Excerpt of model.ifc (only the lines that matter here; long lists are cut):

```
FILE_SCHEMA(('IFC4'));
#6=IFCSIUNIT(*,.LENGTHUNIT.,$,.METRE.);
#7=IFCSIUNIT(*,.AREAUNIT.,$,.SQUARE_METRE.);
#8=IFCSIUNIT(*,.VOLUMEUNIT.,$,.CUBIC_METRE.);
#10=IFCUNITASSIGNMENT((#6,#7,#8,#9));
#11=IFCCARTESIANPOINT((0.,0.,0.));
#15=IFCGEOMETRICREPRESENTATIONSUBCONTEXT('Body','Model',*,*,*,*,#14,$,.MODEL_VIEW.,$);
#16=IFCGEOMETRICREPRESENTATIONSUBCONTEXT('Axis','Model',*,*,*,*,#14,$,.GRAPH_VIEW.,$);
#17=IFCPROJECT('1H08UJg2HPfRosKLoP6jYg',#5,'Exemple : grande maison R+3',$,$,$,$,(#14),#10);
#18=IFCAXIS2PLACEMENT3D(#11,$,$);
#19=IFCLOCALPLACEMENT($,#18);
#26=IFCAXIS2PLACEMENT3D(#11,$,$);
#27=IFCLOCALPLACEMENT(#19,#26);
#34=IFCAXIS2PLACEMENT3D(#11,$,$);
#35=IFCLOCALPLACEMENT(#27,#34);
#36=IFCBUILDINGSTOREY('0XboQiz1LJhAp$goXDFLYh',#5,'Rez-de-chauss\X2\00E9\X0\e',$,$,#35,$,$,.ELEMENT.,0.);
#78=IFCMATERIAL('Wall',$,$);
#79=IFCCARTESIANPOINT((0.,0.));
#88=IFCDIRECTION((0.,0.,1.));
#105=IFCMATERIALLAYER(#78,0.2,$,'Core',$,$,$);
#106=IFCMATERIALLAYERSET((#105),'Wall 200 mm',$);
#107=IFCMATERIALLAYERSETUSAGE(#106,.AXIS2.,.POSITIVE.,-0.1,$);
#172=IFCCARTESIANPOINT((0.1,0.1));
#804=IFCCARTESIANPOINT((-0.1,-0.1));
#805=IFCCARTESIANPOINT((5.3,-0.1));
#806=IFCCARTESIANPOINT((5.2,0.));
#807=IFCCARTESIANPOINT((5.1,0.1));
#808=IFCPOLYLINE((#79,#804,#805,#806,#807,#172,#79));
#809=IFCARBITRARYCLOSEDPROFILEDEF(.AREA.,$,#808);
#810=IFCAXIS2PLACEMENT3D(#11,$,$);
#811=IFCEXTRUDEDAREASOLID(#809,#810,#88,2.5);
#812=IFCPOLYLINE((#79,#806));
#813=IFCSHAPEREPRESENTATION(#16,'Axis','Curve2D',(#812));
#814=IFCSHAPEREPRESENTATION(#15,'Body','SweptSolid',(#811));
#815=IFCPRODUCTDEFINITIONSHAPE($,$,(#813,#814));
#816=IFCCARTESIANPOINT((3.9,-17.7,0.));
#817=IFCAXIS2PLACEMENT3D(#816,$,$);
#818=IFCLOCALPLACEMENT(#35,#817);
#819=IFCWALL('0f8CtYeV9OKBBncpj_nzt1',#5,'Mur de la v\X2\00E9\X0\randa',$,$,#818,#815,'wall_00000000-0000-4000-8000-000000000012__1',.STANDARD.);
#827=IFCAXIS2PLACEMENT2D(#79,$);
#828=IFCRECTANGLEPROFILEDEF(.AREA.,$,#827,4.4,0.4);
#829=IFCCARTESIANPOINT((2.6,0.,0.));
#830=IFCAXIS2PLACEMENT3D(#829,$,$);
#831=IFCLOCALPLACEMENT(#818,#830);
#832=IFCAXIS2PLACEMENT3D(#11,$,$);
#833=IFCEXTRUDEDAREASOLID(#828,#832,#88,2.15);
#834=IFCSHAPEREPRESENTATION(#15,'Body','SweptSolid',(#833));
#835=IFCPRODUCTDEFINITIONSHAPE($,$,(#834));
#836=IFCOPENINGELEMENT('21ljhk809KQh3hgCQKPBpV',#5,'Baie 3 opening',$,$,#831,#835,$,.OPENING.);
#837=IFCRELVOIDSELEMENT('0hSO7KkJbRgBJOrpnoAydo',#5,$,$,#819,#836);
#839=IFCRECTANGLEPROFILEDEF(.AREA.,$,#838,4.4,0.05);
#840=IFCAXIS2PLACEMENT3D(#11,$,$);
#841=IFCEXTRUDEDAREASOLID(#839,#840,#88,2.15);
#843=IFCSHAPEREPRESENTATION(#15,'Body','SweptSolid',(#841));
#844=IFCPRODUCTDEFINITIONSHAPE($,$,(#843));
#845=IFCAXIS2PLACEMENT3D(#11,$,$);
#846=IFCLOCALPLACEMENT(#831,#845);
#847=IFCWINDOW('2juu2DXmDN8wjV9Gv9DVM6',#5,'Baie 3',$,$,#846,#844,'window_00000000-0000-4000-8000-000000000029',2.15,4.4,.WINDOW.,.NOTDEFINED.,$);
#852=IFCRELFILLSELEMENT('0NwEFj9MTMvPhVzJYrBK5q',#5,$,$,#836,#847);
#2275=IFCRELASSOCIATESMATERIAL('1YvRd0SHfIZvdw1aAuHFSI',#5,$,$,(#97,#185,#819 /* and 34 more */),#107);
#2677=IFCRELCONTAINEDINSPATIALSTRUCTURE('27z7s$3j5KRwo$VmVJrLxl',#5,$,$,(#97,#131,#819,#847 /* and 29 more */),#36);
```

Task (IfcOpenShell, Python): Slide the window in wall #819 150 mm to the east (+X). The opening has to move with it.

```python
import ifcopenshell
import ifcopenshell.api.geometry
import ifcopenshell.util.placement
import ifcopenshell.util.unit

model = ifcopenshell.open("model.ifc")
unit_scale = ifcopenshell.util.unit.calculate_unit_scale(model)

window = model.by_id(847)
opening = window.FillsVoids[0].RelatingOpeningElement
wall = opening.VoidsElements[0].RelatingBuildingElement

wall_matrix = ifcopenshell.util.placement.get_local_placement(wall.ObjectPlacement)
shift = wall_matrix[:3, 0] * 0.15 / unit_scale
before = ifcopenshell.util.placement.get_local_placement(window.ObjectPlacement)[:3, 3].copy()

# The window is placed relative to its opening, so it follows when the opening moves.
matrix = ifcopenshell.util.placement.get_local_placement(opening.ObjectPlacement)
matrix[:3, 3] += shift
ifcopenshell.api.geometry.edit_object_placement(
    model, product=opening, matrix=matrix, is_si=False, should_transform_children=True
)

after = ifcopenshell.util.placement.get_local_placement(window.ObjectPlacement)[:3, 3]
print("window moved by", (after - before).round(3) + 0.0)

model.write("model-out.ifc")
```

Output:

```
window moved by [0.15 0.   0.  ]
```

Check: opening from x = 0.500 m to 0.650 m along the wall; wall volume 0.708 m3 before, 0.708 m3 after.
